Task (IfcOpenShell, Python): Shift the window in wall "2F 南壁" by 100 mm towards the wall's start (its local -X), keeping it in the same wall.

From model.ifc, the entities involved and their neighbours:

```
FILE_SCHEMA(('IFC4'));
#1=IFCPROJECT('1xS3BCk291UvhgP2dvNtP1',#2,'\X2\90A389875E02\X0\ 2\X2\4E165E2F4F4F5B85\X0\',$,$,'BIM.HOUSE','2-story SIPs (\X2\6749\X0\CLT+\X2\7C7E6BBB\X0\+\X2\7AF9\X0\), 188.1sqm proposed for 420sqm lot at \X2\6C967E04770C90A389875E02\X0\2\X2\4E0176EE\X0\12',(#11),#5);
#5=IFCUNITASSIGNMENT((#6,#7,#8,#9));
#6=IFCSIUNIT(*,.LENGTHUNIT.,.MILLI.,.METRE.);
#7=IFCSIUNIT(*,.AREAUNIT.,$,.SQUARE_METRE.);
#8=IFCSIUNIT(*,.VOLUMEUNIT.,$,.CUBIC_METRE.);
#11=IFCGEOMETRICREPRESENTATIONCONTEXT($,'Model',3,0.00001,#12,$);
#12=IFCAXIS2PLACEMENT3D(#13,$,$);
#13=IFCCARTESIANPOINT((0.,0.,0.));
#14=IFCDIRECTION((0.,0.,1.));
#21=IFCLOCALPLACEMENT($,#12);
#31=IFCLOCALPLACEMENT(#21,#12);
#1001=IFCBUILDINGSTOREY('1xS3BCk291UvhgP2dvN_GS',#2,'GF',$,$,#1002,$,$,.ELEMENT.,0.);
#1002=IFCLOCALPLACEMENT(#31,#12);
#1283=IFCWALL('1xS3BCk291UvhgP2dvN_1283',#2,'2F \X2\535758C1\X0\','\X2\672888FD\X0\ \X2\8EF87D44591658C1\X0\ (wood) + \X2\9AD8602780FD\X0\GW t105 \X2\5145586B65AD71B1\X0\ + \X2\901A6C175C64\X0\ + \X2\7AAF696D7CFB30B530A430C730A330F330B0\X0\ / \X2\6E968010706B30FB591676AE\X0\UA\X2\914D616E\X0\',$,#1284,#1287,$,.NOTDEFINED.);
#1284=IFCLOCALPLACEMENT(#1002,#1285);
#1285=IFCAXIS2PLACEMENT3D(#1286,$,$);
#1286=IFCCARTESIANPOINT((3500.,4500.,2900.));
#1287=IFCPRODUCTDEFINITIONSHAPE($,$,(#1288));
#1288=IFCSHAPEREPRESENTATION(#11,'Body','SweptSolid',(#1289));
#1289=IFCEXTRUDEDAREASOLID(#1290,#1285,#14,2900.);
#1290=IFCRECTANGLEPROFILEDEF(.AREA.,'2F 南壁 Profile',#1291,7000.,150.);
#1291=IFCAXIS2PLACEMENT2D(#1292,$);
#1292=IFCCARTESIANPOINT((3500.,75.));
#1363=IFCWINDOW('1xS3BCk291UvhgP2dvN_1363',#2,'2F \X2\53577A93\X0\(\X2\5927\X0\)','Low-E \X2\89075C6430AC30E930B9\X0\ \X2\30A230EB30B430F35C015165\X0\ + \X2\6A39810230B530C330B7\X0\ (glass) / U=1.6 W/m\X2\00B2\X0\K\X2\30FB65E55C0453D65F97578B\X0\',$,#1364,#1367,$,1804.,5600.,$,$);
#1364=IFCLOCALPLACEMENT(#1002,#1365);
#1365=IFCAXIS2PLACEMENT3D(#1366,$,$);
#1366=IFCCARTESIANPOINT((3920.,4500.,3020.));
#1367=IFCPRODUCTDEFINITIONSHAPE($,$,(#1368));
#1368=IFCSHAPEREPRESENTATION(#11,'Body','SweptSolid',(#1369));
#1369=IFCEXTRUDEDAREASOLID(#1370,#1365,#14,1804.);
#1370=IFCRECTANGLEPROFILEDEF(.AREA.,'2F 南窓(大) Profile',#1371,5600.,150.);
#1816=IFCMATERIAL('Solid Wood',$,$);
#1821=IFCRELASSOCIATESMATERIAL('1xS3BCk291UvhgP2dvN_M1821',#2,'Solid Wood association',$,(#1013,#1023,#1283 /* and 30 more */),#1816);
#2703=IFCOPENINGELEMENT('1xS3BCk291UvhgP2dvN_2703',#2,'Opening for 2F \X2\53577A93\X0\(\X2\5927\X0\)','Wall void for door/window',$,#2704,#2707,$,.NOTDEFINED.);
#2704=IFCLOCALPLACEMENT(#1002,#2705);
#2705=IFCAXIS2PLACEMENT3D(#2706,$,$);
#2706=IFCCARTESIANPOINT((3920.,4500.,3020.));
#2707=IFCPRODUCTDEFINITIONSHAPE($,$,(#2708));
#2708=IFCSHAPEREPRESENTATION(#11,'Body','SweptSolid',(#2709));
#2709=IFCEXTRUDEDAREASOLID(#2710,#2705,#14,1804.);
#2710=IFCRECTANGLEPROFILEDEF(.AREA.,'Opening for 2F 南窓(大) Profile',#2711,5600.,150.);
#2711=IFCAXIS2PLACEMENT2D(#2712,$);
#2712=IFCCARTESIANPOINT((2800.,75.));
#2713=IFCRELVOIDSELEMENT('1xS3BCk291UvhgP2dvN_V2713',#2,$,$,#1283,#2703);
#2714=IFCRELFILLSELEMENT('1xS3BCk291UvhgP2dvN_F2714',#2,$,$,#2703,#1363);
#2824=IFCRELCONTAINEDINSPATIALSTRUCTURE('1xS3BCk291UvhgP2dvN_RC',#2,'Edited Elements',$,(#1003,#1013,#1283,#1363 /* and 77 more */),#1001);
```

```python
import ifcopenshell
import ifcopenshell.api.geometry
import ifcopenshell.util.placement

model = ifcopenshell.open("model.ifc")

window = model.by_guid("1xS3BCk291UvhgP2dvN_1363")
opening = window.FillsVoids[0].RelatingOpeningElement
wall = opening.VoidsElements[0].RelatingBuildingElement

wall_matrix = ifcopenshell.util.placement.get_local_placement(wall.ObjectPlacement)
shift = wall_matrix[:3, 0] * -100.0
before = ifcopenshell.util.placement.get_local_placement(window.ObjectPlacement)[:3, 3].copy()

# The window is not placed relative to its opening, so move both.
for product in (opening, window):
    matrix = ifcopenshell.util.placement.get_local_placement(product.ObjectPlacement)
    matrix[:3, 3] += shift
    ifcopenshell.api.geometry.edit_object_placement(model, product=product, matrix=matrix, is_si=False)

after = ifcopenshell.util.placement.get_local_placement(window.ObjectPlacement)[:3, 3]
print("window moved by", (after - before).round(3) + 0.0)

model.write("model_v2.ifc")
```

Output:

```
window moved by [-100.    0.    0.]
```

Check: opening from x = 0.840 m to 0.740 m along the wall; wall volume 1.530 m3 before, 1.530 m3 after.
